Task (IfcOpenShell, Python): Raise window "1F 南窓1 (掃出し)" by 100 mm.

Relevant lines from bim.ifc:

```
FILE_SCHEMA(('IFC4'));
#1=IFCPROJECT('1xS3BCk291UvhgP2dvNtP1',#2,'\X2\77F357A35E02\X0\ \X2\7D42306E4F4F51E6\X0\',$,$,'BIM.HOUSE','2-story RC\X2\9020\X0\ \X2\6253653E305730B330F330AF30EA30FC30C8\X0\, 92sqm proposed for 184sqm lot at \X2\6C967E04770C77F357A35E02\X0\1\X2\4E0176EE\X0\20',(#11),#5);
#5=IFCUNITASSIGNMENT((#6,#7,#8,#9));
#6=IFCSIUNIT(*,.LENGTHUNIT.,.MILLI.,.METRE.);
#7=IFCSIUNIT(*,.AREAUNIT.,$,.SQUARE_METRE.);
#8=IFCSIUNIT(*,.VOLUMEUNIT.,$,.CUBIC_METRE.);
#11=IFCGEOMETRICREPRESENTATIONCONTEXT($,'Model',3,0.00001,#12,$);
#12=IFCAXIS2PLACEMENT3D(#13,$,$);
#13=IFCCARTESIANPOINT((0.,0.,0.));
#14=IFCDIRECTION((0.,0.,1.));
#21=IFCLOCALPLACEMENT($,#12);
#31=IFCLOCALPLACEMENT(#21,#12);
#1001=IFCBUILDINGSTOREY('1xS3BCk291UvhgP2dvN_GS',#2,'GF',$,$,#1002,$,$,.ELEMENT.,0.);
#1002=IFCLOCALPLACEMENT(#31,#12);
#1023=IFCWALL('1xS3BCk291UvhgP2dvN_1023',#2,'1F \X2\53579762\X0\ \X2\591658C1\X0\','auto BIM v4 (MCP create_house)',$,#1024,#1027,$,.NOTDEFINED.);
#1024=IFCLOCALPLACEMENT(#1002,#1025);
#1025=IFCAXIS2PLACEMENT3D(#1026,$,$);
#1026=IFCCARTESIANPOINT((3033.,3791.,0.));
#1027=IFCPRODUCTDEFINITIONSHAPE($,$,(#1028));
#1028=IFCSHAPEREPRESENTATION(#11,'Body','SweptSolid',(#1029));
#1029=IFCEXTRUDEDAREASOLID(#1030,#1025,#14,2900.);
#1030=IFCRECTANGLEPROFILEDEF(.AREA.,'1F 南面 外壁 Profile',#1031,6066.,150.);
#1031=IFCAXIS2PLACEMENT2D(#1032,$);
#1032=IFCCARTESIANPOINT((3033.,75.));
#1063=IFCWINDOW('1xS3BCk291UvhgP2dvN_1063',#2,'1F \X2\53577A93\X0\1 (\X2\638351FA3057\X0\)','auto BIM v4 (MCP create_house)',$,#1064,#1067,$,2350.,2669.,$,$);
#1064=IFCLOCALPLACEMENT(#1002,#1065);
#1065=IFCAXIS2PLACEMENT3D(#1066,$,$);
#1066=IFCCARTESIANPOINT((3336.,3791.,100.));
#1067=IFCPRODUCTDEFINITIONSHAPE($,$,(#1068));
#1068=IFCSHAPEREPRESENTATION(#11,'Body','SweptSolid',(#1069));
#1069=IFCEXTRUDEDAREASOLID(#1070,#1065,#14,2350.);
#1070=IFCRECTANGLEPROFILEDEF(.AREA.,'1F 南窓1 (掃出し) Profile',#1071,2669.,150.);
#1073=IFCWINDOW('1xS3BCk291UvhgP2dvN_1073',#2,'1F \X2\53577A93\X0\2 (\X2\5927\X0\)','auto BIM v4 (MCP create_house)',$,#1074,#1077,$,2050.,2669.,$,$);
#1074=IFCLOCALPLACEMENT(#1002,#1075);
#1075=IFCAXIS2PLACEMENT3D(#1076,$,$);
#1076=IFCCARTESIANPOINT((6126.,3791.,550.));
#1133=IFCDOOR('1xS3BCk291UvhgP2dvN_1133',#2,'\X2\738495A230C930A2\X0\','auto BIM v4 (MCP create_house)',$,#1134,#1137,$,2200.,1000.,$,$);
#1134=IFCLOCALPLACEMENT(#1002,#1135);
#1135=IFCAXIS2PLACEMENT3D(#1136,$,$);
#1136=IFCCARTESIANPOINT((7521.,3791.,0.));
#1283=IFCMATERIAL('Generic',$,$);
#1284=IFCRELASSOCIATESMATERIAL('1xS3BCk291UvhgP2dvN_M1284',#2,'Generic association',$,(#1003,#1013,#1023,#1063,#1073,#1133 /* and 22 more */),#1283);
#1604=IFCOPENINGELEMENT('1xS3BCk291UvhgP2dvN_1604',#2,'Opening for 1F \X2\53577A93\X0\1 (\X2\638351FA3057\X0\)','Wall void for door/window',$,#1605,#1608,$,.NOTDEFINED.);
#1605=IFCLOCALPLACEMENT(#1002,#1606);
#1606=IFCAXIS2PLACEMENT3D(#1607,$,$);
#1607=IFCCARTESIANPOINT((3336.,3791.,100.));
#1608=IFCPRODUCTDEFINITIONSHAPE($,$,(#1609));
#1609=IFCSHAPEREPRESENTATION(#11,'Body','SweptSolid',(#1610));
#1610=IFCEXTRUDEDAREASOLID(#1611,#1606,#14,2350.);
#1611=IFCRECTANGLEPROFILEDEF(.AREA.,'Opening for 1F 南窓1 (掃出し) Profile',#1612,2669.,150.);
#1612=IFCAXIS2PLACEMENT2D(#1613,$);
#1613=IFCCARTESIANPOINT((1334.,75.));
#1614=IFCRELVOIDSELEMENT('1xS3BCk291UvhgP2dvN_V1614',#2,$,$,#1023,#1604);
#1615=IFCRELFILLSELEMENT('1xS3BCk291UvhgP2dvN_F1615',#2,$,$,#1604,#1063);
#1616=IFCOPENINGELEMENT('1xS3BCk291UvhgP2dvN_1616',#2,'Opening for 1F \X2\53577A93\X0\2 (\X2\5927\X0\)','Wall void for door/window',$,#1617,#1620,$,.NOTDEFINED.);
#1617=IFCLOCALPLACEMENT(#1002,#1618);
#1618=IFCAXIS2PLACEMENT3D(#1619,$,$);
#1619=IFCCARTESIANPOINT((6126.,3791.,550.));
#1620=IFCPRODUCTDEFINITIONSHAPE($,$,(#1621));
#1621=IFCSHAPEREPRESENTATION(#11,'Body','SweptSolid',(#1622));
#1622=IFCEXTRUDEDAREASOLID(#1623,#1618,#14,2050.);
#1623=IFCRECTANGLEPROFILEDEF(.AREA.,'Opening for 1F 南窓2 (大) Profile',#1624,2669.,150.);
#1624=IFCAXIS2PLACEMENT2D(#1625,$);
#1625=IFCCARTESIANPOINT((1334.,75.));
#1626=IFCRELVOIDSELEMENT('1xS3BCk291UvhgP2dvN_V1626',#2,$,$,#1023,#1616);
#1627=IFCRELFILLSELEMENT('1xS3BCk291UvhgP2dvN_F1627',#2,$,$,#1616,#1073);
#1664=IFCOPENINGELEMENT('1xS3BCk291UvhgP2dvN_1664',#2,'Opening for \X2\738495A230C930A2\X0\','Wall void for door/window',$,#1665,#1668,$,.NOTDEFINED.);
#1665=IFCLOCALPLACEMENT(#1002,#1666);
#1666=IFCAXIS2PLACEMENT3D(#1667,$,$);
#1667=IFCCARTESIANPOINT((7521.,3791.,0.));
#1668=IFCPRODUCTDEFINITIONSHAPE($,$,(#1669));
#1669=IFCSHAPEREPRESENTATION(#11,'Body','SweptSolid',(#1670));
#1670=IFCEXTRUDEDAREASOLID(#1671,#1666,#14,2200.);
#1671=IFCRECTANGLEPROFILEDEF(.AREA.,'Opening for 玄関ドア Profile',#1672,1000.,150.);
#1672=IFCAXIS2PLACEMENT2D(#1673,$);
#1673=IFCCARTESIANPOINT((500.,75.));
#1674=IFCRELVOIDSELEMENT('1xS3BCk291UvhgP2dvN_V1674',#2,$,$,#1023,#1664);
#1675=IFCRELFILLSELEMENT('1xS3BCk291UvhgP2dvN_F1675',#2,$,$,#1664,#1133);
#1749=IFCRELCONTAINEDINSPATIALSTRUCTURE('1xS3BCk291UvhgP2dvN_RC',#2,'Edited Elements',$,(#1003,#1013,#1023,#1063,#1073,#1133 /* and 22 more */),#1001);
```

```python
import numpy as np
import ifcopenshell
import ifcopenshell.api.geometry
import ifcopenshell.util.placement
import ifcopenshell.util.unit

model = ifcopenshell.open("bim.ifc")
unit_scale = ifcopenshell.util.unit.calculate_unit_scale(model)

window = model.by_guid("1xS3BCk291UvhgP2dvN_1063")
opening = window.FillsVoids[0].RelatingOpeningElement
dz = 100.0

shift = np.array([0.0, 0.0, dz])
# The window is not placed relative to its opening, so move both.
for product in (opening, window):
    matrix = ifcopenshell.util.placement.get_local_placement(product.ObjectPlacement)
    matrix[:3, 3] += shift
    ifcopenshell.api.geometry.edit_object_placement(model, product=product, matrix=matrix, is_si=False)

print(f"moved by {dz * unit_scale:+.3f} m")

model.write("bim-out.ifc")
```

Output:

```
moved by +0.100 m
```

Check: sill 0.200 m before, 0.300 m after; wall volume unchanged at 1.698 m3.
